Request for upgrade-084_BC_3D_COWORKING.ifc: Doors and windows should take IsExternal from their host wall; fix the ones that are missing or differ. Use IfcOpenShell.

First a look at what the model holds.

```python
import ifcopenshell
import ifcopenshell.util.element

model = ifcopenshell.open("upgrade-084_BC_3D_COWORKING.ifc")
print(model.schema)
seen = {}
for e in model.by_type("IfcDoor") + model.by_type("IfcWindow"):
    if not e.FillsVoids:
        continue
    host = e.FillsVoids[0].RelatingOpeningElement.VoidsElements[0].RelatingBuildingElement
    own = ifcopenshell.util.element.get_pset(e, f"Pset_{e.is_a()[3:].removesuffix('StandardCase')}Common", "IsExternal")
    wall = ifcopenshell.util.element.get_pset(host, "Pset_WallCommon", "IsExternal")
    seen[e.is_a(), own, wall] = seen.get((e.is_a(), own, wall), 0) + 1
for (cls, own, wall), count in sorted(seen.items(), key=str):
    print(count, cls, "IsExternal:", own, "| host wall:", wall)
```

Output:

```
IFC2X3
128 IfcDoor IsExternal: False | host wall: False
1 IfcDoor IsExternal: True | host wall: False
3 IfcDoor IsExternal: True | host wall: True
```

```python
import ifcopenshell
import ifcopenshell.api.pset
import ifcopenshell.util.element

model = ifcopenshell.open("upgrade-084_BC_3D_COWORKING.ifc")

count = 0
for ifc_class, pset_name in (("IfcDoor", "Pset_DoorCommon"), ("IfcWindow", "Pset_WindowCommon")):
    for e in model.by_type(ifc_class):
        if not e.FillsVoids:
            continue
        host = e.FillsVoids[0].RelatingOpeningElement.VoidsElements[0].RelatingBuildingElement
        external = ifcopenshell.util.element.get_pset(host, "Pset_WallCommon", "IsExternal")
        if external is None or ifcopenshell.util.element.get_pset(e, pset_name, "IsExternal") == external:
            continue
        pset = ifcopenshell.api.pset.add_pset(model, product=e, name=pset_name)
        ifcopenshell.api.pset.edit_pset(model, pset=pset, properties={"IsExternal": external})
        count += 1

print(count, "updated")

model.write("upgrade-084_BC_3D_COWORKING_edited.ifc")
```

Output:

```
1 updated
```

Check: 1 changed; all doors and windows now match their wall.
